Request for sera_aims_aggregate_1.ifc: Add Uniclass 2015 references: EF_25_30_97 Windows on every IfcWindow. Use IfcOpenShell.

First a look at what the model holds.

```python
import ifcopenshell

model = ifcopenshell.open("sera_aims_aggregate_1.ifc")
print(model.schema)
print("classifications:", [c.Name for c in model.by_type("IfcClassification")])
for ifc_class in ("IfcDoor", "IfcRoof", "IfcStair", "IfcWall", "IfcWindow"):
    print(ifc_class, len(model.by_type(ifc_class)))
```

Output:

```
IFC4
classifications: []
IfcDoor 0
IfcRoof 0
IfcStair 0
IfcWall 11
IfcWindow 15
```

```python
import ifcopenshell
import ifcopenshell.api.classification

model = ifcopenshell.open("sera_aims_aggregate_1.ifc")

system = ifcopenshell.api.classification.add_classification(model, classification="Uniclass 2015")

codes = {
    "IfcWindow": ("EF_25_30_97", "Windows"),
}
for ifc_class, (code, name) in codes.items():
    products = model.by_type(ifc_class)
    ifcopenshell.api.classification.add_reference(
        model, products=products, classification=system, identification=code, name=name
    )
    print(code, len(products))

model.write("sera_aims_aggregate_1_v2.ifc")
```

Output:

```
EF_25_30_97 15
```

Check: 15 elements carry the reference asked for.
